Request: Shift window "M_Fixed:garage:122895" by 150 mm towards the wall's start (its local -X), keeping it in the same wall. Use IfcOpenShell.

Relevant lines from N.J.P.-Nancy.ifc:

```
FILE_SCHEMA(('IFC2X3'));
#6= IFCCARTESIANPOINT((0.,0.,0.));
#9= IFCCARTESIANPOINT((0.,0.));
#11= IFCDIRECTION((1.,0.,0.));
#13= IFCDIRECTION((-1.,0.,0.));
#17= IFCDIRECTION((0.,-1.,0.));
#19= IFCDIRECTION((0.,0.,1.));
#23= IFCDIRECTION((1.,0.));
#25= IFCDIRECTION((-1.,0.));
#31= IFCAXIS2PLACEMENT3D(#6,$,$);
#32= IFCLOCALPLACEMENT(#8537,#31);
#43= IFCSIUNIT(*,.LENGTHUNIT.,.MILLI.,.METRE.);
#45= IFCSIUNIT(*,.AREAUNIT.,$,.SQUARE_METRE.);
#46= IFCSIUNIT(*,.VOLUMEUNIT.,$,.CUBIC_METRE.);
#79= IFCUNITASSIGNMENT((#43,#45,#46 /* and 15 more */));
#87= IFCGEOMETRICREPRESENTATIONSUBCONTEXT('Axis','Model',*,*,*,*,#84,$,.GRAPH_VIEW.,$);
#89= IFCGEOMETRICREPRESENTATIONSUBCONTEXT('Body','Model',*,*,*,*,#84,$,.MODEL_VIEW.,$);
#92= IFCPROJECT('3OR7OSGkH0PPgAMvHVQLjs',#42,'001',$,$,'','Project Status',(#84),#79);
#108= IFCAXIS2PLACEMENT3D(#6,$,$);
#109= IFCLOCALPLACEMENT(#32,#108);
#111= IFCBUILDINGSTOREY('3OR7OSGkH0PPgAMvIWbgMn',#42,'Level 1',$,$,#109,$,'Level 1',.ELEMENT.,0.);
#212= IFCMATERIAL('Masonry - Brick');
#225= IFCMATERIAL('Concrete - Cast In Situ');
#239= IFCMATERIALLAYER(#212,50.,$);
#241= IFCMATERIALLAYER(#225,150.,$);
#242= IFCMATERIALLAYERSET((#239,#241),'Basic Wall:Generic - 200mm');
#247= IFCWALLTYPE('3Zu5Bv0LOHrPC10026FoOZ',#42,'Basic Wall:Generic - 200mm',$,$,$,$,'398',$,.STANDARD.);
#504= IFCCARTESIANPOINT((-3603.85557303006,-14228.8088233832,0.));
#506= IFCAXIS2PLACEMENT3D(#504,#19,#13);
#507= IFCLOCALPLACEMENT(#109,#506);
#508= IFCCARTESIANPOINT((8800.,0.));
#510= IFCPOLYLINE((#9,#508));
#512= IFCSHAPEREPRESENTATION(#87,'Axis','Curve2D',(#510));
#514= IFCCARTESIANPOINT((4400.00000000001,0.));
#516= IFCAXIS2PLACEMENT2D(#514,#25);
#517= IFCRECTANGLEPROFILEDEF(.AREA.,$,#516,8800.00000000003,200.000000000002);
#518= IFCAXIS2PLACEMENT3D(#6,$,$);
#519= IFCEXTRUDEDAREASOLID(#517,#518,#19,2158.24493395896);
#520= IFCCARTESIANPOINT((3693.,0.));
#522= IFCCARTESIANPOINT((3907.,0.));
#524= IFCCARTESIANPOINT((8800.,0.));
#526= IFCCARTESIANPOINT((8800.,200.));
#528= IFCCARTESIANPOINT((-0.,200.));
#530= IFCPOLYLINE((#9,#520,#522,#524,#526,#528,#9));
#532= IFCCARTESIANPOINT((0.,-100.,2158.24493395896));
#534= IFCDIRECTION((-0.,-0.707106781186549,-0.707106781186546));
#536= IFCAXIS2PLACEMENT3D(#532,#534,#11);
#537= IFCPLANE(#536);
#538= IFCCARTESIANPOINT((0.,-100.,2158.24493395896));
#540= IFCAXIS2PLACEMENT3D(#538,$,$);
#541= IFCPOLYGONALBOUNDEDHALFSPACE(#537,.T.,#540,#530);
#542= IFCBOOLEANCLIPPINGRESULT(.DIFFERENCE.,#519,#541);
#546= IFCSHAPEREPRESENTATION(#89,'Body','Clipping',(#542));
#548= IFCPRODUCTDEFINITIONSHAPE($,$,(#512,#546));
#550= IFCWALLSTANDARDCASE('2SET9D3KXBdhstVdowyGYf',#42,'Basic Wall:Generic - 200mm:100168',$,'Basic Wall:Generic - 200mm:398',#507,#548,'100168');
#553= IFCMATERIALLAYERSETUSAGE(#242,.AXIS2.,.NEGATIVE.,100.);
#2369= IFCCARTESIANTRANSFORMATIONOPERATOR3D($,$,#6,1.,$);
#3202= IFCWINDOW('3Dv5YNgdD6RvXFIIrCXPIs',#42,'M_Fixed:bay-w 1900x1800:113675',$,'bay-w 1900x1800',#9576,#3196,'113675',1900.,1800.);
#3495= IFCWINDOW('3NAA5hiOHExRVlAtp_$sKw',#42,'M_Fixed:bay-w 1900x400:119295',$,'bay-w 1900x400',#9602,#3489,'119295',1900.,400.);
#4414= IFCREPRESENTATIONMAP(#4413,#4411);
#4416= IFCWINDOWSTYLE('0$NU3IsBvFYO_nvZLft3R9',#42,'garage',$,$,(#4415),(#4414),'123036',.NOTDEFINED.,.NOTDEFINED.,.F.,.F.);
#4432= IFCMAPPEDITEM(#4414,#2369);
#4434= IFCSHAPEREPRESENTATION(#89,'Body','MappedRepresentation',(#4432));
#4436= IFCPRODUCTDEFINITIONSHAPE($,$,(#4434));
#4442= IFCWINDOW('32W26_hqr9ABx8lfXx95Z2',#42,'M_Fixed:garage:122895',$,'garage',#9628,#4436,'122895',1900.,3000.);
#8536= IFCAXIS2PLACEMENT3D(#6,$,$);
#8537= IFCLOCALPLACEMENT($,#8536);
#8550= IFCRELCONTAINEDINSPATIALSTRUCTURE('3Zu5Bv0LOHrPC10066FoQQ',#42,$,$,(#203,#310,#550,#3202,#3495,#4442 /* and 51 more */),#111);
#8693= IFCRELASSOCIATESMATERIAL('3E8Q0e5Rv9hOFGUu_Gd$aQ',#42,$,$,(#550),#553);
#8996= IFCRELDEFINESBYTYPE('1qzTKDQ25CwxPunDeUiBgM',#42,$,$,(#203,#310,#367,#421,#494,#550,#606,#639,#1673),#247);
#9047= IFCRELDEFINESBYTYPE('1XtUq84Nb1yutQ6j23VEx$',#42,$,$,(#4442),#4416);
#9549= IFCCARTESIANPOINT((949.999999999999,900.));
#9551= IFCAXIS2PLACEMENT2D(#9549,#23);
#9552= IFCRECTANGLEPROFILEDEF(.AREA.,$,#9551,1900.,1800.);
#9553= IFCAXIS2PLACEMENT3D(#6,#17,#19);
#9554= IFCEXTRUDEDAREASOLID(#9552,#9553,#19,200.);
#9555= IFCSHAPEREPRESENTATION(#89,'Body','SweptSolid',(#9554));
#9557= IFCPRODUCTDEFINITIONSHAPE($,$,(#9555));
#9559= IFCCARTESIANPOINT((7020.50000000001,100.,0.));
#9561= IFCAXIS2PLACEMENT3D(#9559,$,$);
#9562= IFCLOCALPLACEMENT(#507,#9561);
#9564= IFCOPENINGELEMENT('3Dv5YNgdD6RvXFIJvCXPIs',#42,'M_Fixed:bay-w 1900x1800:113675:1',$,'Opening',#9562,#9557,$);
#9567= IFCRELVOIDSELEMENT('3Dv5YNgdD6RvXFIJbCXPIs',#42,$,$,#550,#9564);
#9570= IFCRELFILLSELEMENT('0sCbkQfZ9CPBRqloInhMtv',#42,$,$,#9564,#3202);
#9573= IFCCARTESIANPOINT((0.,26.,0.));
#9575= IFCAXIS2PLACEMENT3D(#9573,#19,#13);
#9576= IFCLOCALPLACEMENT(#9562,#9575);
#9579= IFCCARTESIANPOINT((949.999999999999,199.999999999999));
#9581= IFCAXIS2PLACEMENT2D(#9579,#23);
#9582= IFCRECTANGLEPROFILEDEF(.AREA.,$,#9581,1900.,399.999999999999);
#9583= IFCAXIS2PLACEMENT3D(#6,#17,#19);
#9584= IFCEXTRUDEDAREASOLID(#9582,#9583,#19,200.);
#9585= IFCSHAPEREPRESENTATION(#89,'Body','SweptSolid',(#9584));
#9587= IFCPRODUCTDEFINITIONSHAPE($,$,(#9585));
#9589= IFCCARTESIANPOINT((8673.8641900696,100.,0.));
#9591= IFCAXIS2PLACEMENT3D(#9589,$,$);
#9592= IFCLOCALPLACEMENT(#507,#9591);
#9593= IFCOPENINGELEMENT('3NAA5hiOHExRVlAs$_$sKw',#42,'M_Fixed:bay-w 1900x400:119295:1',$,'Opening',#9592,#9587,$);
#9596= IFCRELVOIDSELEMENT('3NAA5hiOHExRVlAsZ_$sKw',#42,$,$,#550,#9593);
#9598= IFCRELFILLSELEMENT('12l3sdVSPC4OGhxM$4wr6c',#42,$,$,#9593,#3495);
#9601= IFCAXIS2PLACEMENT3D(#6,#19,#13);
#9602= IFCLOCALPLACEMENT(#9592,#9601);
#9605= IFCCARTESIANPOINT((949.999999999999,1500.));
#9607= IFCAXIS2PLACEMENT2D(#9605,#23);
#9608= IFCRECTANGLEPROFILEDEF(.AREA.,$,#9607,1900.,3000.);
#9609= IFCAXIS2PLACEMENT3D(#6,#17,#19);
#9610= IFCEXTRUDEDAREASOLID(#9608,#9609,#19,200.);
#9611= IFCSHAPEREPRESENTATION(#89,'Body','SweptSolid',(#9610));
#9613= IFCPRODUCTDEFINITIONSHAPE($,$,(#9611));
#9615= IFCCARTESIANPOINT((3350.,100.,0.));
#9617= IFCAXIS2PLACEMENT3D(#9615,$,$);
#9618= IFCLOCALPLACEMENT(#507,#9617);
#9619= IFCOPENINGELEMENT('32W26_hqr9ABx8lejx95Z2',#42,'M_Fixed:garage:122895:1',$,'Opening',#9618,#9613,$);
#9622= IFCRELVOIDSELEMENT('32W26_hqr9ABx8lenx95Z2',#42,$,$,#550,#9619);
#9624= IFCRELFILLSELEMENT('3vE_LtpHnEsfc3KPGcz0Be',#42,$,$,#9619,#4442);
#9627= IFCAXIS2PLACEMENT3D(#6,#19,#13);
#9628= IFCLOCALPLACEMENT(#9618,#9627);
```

```python
import ifcopenshell
import ifcopenshell.api.geometry
import ifcopenshell.util.placement

model = ifcopenshell.open("N.J.P.-Nancy.ifc")

window = model.by_guid("32W26_hqr9ABx8lfXx95Z2")
opening = window.FillsVoids[0].RelatingOpeningElement
wall = opening.VoidsElements[0].RelatingBuildingElement

wall_matrix = ifcopenshell.util.placement.get_local_placement(wall.ObjectPlacement)
shift = wall_matrix[:3, 0] * -150.0
before = ifcopenshell.util.placement.get_local_placement(window.ObjectPlacement)[:3, 3].copy()

# The window is placed relative to its opening, so it follows when the opening moves.
matrix = ifcopenshell.util.placement.get_local_placement(opening.ObjectPlacement)
matrix[:3, 3] += shift
ifcopenshell.api.geometry.edit_object_placement(
    model, product=opening, matrix=matrix, is_si=False, should_transform_children=True
)

after = ifcopenshell.util.placement.get_local_placement(window.ObjectPlacement)[:3, 3]
print("window moved by", (after - before).round(3) + 0.0)

model.write("N.J.P.-Nancy_updated.ifc")
```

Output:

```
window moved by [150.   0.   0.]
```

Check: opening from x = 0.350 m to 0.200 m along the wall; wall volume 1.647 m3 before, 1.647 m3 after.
